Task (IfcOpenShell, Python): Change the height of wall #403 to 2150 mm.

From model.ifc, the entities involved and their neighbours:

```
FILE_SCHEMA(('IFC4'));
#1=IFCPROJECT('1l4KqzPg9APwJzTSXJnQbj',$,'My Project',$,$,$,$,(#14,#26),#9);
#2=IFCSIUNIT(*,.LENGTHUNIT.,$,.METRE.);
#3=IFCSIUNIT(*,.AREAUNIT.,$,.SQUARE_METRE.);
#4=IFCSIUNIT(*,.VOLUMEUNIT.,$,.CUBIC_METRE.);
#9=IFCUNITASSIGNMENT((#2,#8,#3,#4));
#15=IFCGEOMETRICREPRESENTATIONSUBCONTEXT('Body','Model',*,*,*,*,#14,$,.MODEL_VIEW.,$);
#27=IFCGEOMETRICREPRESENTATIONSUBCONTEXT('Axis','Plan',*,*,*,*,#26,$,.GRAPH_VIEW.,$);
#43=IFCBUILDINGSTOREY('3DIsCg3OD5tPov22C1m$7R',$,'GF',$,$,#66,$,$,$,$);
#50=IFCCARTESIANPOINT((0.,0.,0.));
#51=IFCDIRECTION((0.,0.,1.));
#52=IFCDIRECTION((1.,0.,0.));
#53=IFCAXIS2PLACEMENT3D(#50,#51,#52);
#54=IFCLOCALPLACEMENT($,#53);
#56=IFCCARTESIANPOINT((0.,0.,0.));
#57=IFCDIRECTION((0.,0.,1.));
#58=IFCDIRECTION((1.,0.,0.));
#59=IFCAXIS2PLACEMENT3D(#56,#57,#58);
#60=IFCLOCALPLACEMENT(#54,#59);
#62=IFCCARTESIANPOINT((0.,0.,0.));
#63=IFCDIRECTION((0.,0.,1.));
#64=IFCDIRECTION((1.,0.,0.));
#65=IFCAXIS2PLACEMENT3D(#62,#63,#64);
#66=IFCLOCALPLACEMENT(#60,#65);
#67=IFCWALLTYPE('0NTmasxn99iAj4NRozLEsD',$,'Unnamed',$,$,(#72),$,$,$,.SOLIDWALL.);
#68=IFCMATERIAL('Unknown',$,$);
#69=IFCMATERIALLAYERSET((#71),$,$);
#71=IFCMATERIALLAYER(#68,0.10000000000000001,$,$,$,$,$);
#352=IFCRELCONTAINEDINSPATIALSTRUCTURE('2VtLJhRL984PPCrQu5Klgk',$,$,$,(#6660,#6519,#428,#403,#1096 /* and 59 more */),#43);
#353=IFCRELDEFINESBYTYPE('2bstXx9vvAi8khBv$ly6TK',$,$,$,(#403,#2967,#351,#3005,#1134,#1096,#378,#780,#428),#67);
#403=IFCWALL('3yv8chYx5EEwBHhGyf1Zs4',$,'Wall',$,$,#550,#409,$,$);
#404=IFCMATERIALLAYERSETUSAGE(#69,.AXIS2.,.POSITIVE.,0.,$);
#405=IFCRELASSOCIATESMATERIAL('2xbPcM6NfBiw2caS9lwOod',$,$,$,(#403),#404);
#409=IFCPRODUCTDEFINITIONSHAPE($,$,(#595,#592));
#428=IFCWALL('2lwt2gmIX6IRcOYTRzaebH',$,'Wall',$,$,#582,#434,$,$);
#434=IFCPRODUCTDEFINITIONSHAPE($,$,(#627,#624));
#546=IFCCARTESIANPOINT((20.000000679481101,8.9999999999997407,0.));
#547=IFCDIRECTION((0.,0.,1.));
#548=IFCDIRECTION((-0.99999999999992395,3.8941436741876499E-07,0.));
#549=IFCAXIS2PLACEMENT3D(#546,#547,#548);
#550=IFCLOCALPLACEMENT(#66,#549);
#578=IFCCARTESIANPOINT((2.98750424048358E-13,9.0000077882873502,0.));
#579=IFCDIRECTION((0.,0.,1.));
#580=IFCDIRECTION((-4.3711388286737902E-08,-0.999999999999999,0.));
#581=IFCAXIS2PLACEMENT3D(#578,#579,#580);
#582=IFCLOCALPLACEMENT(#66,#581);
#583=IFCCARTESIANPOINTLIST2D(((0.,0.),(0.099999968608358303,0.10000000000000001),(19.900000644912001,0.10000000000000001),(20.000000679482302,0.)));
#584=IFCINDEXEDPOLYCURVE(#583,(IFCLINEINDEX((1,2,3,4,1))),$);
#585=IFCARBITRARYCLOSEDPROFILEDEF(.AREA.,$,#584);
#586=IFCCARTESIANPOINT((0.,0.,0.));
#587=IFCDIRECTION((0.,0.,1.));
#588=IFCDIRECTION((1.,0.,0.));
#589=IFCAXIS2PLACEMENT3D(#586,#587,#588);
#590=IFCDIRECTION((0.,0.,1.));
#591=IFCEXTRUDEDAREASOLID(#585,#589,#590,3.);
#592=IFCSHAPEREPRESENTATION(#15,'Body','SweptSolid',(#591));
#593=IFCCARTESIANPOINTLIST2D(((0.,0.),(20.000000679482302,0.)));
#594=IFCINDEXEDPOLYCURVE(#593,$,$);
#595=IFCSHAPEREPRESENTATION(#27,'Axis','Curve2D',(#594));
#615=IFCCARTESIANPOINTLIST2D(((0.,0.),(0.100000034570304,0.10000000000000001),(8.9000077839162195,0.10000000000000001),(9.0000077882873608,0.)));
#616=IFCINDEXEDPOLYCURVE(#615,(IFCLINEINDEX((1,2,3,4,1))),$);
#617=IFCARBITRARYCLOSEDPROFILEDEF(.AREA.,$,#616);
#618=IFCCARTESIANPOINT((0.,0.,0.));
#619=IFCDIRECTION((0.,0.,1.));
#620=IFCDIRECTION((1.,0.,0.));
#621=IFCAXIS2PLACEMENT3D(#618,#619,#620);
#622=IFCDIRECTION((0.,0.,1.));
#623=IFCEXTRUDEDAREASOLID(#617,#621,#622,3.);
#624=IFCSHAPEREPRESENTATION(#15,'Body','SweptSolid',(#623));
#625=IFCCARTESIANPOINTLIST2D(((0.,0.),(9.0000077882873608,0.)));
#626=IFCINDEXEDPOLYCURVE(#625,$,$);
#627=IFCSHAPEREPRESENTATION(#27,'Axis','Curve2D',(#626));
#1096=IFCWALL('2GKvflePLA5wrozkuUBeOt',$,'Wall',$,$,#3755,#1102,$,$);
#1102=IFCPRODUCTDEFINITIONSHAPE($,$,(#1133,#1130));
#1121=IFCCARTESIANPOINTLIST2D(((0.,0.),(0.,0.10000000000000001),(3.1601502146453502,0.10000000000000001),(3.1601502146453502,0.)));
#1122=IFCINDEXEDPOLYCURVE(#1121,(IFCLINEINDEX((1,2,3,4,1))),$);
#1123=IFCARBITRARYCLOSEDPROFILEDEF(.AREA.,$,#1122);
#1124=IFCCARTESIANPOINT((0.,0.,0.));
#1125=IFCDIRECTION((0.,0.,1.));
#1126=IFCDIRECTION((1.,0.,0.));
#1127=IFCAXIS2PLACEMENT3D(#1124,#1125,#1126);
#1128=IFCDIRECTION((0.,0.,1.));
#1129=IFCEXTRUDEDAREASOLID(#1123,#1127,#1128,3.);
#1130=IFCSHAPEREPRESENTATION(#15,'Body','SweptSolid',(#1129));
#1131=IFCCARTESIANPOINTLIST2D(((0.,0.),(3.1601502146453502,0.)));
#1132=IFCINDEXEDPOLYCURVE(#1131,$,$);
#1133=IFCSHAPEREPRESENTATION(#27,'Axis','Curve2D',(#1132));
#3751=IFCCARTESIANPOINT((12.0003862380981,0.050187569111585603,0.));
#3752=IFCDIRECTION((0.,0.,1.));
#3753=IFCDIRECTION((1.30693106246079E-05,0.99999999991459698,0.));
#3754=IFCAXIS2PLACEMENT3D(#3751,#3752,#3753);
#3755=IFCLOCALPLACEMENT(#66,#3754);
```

```python
import ifcopenshell
import ifcopenshell.geom
import ifcopenshell.util.representation
import ifcopenshell.util.shape
import ifcopenshell.util.unit

model = ifcopenshell.open("model.ifc")
unit_scale = ifcopenshell.util.unit.calculate_unit_scale(model)
settings = ifcopenshell.geom.settings()


def volume(element):
    """Net volume in cubic metres, openings subtracted."""
    shape = ifcopenshell.geom.create_shape(settings, element)
    return ifcopenshell.util.shape.get_volume(shape.geometry)


wall = model.by_guid("3yv8chYx5EEwBHhGyf1Zs4")
before = volume(wall)

body = ifcopenshell.util.representation.get_representation(wall, "Model", "Body")
solid = body.Items[0]
old_height = solid.Depth
solid.Depth = 2.15 / unit_scale
after = volume(wall)

print(f"height {old_height:g} -> {solid.Depth:g}, volume {before:.3f} -> {after:.3f} m3")

model.write("model_updated.ifc")
```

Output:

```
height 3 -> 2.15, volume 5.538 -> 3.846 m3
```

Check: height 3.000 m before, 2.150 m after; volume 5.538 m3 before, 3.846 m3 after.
